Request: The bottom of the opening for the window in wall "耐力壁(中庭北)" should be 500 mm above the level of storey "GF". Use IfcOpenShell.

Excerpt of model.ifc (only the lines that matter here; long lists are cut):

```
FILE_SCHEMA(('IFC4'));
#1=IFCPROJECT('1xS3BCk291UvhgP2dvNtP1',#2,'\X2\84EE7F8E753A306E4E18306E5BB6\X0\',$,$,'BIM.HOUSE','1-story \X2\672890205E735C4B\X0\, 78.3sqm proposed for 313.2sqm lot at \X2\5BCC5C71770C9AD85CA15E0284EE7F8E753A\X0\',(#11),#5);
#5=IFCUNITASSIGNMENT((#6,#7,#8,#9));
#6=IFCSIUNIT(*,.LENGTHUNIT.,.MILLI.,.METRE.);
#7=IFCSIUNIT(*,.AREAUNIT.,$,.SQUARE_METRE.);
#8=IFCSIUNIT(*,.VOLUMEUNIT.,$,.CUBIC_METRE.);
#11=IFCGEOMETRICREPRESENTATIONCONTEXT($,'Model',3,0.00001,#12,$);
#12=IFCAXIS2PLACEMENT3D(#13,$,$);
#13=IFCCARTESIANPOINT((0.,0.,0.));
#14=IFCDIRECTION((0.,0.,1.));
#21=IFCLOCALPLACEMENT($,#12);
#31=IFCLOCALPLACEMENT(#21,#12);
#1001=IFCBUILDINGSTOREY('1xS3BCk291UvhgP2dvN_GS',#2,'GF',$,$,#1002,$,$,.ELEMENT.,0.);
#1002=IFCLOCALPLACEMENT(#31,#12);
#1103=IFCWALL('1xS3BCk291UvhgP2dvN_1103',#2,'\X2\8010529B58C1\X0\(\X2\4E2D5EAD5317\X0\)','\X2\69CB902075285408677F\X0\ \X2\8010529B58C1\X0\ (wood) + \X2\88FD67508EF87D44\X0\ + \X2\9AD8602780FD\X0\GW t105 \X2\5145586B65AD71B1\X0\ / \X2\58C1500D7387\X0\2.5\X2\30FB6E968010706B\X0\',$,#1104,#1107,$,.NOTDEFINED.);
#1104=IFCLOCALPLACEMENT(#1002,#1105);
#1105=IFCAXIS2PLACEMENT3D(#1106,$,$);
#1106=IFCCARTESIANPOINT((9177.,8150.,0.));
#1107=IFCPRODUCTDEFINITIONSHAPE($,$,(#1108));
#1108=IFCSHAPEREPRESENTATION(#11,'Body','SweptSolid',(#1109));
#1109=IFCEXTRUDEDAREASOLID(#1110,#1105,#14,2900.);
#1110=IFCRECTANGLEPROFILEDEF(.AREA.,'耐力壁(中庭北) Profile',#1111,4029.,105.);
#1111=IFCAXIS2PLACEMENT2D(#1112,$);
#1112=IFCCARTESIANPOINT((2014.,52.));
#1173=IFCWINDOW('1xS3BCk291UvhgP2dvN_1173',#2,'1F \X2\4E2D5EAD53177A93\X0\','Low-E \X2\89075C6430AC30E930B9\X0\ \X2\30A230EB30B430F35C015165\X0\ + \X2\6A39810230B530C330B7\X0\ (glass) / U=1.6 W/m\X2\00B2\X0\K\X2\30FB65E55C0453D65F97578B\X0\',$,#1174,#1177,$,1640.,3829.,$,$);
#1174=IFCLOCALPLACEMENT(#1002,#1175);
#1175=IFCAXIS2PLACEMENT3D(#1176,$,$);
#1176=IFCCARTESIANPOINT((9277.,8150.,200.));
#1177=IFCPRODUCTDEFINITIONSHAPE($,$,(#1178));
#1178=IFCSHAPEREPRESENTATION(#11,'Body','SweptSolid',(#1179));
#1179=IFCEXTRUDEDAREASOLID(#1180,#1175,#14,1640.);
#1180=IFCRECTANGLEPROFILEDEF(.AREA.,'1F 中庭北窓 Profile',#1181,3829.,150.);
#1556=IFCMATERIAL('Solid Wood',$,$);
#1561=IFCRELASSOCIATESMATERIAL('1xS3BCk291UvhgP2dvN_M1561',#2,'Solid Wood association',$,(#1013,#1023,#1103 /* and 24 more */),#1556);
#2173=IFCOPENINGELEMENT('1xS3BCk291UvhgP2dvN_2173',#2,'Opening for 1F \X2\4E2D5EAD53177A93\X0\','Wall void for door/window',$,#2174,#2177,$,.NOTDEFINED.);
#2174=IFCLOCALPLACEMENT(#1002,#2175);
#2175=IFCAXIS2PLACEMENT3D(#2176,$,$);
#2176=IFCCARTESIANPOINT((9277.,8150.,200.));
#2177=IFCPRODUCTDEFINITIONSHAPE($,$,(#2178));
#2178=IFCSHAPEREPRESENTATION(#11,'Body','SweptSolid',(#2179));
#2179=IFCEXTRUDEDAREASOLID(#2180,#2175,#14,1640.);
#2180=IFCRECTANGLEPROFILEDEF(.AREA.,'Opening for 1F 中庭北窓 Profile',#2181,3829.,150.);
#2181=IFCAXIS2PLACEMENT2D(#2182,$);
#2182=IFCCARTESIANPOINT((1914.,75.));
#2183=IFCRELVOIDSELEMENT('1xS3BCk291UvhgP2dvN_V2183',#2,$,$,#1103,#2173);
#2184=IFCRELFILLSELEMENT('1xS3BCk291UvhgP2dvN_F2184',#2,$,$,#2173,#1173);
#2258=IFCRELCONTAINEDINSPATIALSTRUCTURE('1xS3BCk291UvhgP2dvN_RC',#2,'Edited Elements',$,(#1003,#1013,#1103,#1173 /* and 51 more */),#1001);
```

```python
import numpy as np
import ifcopenshell
import ifcopenshell.api.geometry
import ifcopenshell.geom
import ifcopenshell.util.element
import ifcopenshell.util.placement
import ifcopenshell.util.shape
import ifcopenshell.util.unit

model = ifcopenshell.open("model.ifc")
unit_scale = ifcopenshell.util.unit.calculate_unit_scale(model)

window = model.by_id(1173)
opening = window.FillsVoids[0].RelatingOpeningElement
storey = ifcopenshell.util.element.get_container(window, ifc_class="IfcBuildingStorey")
level = ifcopenshell.util.placement.get_local_placement(storey.ObjectPlacement)[2, 3]

# The opening's origin need not be at the sill, so measure its lowest point.
shape = ifcopenshell.geom.create_shape(ifcopenshell.geom.settings(), opening)
bottom = ifcopenshell.util.shape.get_shape_bottom_elevation(shape, shape.geometry) / unit_scale
dz = level + 0.5 / unit_scale - bottom

shift = np.array([0.0, 0.0, dz])
# The window is not placed relative to its opening, so move both.
for product in (opening, window):
    matrix = ifcopenshell.util.placement.get_local_placement(product.ObjectPlacement)
    matrix[:3, 3] += shift
    ifcopenshell.api.geometry.edit_object_placement(model, product=product, matrix=matrix, is_si=False)

print(f"moved by {dz * unit_scale:+.3f} m")

model.write("model-out.ifc")
```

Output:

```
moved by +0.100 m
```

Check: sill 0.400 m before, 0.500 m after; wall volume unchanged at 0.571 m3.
